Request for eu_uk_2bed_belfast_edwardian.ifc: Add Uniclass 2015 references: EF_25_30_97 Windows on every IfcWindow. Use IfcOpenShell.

First a look at what the model holds.

```python
import ifcopenshell

model = ifcopenshell.open("eu_uk_2bed_belfast_edwardian.ifc")
print(model.schema)
print("classifications:", [c.Name for c in model.by_type("IfcClassification")])
for ifc_class in ("IfcDoor", "IfcRoof", "IfcStair", "IfcWall", "IfcWindow"):
    print(ifc_class, len(model.by_type(ifc_class)))
```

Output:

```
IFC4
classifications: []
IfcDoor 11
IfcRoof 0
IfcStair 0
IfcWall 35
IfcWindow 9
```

```python
import ifcopenshell
import ifcopenshell.api.classification

model = ifcopenshell.open("eu_uk_2bed_belfast_edwardian.ifc")

system = ifcopenshell.api.classification.add_classification(model, classification="Uniclass 2015")

codes = {
    "IfcWindow": ("EF_25_30_97", "Windows"),
}
for ifc_class, (code, name) in codes.items():
    products = model.by_type(ifc_class)
    ifcopenshell.api.classification.add_reference(
        model, products=products, classification=system, identification=code, name=name
    )
    print(code, len(products))

model.write("eu_uk_2bed_belfast_edwardian_v2.ifc")
```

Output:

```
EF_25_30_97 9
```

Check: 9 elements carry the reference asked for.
